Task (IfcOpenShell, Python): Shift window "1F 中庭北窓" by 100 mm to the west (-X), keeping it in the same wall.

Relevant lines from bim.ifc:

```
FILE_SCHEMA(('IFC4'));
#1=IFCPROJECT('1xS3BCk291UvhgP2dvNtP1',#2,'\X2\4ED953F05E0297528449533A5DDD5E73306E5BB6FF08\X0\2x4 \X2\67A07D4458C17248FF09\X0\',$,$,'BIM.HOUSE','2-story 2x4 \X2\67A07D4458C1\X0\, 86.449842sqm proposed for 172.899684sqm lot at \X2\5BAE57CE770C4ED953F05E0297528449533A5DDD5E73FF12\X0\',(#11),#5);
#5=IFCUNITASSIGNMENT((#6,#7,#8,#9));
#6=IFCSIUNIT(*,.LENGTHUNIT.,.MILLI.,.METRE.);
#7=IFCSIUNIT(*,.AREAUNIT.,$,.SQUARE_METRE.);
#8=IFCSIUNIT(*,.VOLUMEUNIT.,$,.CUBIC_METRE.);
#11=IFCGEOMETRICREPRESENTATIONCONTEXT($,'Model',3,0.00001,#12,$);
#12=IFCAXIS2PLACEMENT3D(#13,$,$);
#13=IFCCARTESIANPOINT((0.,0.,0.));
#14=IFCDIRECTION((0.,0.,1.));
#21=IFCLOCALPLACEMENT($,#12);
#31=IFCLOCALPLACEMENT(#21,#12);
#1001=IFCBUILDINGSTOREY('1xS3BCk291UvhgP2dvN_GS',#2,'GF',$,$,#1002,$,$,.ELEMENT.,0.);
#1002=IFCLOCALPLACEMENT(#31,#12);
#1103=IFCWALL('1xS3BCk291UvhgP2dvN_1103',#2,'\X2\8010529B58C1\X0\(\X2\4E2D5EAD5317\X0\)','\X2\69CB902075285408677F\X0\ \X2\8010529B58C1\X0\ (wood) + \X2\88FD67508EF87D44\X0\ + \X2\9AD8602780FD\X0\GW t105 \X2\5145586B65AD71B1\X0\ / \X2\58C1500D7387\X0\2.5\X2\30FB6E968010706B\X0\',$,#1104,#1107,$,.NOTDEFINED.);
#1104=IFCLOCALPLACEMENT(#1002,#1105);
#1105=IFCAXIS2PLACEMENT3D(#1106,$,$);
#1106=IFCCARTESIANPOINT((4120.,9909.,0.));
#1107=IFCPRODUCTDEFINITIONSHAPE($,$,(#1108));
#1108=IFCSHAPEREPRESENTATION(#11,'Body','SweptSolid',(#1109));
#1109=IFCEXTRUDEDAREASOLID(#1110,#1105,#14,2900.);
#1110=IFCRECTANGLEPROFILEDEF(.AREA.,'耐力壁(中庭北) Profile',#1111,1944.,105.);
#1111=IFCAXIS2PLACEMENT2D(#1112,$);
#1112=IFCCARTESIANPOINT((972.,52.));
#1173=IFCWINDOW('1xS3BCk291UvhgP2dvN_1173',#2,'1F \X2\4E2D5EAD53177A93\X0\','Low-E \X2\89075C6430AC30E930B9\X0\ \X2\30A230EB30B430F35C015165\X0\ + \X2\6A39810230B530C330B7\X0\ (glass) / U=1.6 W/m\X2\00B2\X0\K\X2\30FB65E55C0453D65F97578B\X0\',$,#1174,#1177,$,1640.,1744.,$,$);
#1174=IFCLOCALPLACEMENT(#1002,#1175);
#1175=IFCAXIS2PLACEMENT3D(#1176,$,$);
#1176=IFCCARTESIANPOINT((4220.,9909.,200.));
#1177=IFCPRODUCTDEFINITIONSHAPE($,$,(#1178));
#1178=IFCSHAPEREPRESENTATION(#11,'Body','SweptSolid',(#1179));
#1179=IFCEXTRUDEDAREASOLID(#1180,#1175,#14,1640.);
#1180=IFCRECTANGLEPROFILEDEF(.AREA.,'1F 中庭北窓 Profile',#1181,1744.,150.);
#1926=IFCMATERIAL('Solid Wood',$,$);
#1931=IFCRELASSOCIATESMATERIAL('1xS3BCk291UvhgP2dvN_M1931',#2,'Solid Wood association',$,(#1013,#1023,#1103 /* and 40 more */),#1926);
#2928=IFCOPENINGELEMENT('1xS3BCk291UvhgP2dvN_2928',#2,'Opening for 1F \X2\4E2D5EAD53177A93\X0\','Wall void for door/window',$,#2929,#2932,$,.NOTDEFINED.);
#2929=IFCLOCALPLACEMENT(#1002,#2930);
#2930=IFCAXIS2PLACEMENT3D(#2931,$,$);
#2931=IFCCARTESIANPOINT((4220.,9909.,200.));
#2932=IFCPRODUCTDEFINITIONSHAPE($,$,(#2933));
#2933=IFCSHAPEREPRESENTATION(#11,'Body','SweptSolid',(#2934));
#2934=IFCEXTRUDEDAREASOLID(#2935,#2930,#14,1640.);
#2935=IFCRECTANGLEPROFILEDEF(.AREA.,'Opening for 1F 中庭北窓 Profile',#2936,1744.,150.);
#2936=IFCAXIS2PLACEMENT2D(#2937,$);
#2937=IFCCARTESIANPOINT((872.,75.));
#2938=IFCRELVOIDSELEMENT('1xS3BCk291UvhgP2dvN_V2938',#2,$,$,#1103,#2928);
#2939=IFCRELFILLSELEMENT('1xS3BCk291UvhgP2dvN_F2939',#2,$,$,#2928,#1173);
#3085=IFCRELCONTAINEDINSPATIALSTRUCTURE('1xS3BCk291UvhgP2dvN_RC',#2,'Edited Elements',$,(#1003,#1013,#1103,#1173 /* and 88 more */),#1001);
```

```python
import ifcopenshell
import ifcopenshell.api.geometry
import ifcopenshell.util.placement

model = ifcopenshell.open("bim.ifc")

window = model.by_guid("1xS3BCk291UvhgP2dvN_1173")
opening = window.FillsVoids[0].RelatingOpeningElement
wall = opening.VoidsElements[0].RelatingBuildingElement

wall_matrix = ifcopenshell.util.placement.get_local_placement(wall.ObjectPlacement)
shift = wall_matrix[:3, 0] * -100.0
before = ifcopenshell.util.placement.get_local_placement(window.ObjectPlacement)[:3, 3].copy()

# The window is not placed relative to its opening, so move both.
for product in (opening, window):
    matrix = ifcopenshell.util.placement.get_local_placement(product.ObjectPlacement)
    matrix[:3, 3] += shift
    ifcopenshell.api.geometry.edit_object_placement(model, product=product, matrix=matrix, is_si=False)

after = ifcopenshell.util.placement.get_local_placement(window.ObjectPlacement)[:3, 3]
print("window moved by", (after - before).round(3) + 0.0)

model.write("bim_rev.ifc")
```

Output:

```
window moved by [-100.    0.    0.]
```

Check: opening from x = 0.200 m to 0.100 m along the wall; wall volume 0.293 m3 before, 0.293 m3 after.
